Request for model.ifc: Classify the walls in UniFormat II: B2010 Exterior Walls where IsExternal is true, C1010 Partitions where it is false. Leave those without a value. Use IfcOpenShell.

First a look at what the model holds.

```python
import ifcopenshell
import ifcopenshell.util.element

model = ifcopenshell.open("model.ifc")
print(model.schema)
print("classifications:", [c.Name for c in model.by_type("IfcClassification")])
values = [ifcopenshell.util.element.get_pset(e, "Pset_WallCommon", "IsExternal") for e in model.by_type("IfcWall")]
for value in (True, False, None):
    print("IsExternal", value, values.count(value))
```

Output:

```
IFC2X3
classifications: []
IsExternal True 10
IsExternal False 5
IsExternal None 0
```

```python
import ifcopenshell
import ifcopenshell.api.classification
import ifcopenshell.util.element

model = ifcopenshell.open("model.ifc")

# IFC2X3 requires Source and Edition and has no link from the project to the system.
system = model.create_entity("IfcClassification", Source="ASTM", Edition="E1557", Name="UniFormat II")

walls = model.by_type("IfcWall")
external = {e: ifcopenshell.util.element.get_pset(e, "Pset_WallCommon", "IsExternal") for e in walls}
for flag, code, name in ((True, "B2010", "Exterior Walls"), (False, "C1010", "Partitions")):
    products = [e for e in walls if external[e] is flag]
    ifcopenshell.api.classification.add_reference(
        model, products=products, classification=system, identification=code, name=name
    )
    print(code, len(products))

model.write("model_rev.ifc")
```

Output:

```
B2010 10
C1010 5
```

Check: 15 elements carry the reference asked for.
